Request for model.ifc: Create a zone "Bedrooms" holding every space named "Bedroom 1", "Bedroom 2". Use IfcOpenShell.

First a look at what the model holds.

```python
import ifcopenshell

model = ifcopenshell.open("model.ifc")
print(model.schema)
seen = {}
for space in model.by_type("IfcSpace"):
    seen[space.LongName] = seen.get(space.LongName, 0) + 1
for name, count in sorted(seen.items(), key=str):
    print(count, "x", name)
print("zones:", [z.Name for z in model.by_type("IfcZone")][:20])
```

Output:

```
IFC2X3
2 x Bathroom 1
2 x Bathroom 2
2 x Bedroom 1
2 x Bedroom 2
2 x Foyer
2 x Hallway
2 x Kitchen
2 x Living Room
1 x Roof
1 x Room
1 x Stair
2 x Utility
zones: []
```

```python
import ifcopenshell
import ifcopenshell.api.group
import ifcopenshell.api.root

model = ifcopenshell.open("model.ifc")

names = {"Bedroom 1", "Bedroom 2"}
spaces = [s for s in model.by_type("IfcSpace") if s.LongName in names]

zone = ifcopenshell.api.root.create_entity(model, ifc_class="IfcZone", name="Bedrooms")
ifcopenshell.api.group.assign_group(model, products=spaces, group=zone)
print(len(spaces), "spaces in", zone.Name)

model.write("model_v2.ifc")
```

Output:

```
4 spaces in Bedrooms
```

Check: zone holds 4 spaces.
